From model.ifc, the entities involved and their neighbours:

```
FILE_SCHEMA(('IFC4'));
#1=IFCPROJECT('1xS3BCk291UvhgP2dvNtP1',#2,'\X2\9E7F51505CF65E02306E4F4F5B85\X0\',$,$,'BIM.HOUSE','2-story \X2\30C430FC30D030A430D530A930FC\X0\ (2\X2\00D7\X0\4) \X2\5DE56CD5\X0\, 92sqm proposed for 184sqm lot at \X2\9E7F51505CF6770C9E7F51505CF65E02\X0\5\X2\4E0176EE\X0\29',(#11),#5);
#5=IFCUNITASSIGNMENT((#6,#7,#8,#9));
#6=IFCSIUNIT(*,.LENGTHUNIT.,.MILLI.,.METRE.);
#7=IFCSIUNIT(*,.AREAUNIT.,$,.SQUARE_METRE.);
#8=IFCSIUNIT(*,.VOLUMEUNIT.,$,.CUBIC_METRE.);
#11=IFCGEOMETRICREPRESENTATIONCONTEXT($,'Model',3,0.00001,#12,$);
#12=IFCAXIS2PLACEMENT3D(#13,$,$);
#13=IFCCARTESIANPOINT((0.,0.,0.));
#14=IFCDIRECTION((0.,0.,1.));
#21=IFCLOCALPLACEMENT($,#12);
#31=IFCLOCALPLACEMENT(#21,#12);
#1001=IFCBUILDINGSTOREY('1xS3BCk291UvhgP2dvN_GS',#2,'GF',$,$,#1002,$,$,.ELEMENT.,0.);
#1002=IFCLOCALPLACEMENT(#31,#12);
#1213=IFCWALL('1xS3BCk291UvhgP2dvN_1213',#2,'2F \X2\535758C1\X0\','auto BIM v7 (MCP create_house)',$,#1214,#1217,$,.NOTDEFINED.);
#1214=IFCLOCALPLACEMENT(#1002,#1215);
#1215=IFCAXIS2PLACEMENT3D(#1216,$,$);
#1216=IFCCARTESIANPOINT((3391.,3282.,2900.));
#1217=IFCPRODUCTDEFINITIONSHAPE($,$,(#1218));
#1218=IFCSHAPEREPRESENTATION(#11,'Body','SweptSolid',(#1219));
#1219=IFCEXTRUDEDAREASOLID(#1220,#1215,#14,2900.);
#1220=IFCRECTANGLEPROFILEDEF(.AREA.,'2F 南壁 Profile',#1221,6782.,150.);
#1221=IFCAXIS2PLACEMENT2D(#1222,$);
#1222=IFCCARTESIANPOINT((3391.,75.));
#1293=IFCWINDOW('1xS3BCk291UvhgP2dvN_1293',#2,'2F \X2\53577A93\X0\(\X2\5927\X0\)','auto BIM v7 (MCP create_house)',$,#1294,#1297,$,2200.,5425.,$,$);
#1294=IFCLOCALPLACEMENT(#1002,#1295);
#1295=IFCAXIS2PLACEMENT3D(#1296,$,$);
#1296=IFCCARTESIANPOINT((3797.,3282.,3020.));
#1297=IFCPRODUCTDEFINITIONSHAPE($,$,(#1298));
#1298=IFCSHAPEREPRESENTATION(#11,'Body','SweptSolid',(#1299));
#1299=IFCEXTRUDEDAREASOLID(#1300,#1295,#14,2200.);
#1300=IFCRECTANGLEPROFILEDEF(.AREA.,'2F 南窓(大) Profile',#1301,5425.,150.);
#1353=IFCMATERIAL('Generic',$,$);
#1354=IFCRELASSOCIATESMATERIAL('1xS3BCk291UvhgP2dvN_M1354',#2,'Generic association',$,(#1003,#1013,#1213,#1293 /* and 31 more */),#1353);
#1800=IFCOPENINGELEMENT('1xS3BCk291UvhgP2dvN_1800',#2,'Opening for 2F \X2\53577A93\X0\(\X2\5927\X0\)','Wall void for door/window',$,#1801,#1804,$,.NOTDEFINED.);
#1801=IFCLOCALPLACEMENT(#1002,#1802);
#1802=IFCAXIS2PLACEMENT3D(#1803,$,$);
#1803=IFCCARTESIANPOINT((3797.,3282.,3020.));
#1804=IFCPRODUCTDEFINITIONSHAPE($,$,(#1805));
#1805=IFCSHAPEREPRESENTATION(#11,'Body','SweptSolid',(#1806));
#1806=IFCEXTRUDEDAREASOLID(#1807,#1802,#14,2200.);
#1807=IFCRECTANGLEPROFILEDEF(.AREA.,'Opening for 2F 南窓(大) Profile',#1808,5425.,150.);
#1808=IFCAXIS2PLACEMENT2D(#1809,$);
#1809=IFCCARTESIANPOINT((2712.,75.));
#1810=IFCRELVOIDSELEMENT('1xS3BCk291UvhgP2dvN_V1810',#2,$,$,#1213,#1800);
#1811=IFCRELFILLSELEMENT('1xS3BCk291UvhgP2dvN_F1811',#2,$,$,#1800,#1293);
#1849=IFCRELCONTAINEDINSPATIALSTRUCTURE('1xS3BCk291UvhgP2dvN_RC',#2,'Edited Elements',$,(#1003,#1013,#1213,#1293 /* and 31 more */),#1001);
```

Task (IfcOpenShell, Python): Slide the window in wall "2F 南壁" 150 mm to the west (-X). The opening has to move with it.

```python
import ifcopenshell
import ifcopenshell.api.geometry
import ifcopenshell.util.placement
import ifcopenshell.util.unit

model = ifcopenshell.open("model.ifc")
unit_scale = ifcopenshell.util.unit.calculate_unit_scale(model)

window = model.by_guid("1xS3BCk291UvhgP2dvN_1293")
opening = window.FillsVoids[0].RelatingOpeningElement
wall = opening.VoidsElements[0].RelatingBuildingElement

wall_matrix = ifcopenshell.util.placement.get_local_placement(wall.ObjectPlacement)
shift = wall_matrix[:3, 0] * -0.15 / unit_scale
before = ifcopenshell.util.placement.get_local_placement(window.ObjectPlacement)[:3, 3].copy()

# The window is not placed relative to its opening, so move both.
for product in (opening, window):
    matrix = ifcopenshell.util.placement.get_local_placement(product.ObjectPlacement)
    matrix[:3, 3] += shift
    ifcopenshell.api.geometry.edit_object_placement(model, product=product, matrix=matrix, is_si=False)

after = ifcopenshell.util.placement.get_local_placement(window.ObjectPlacement)[:3, 3]
print("window moved by", (after - before).round(3) + 0.0)

model.write("model_edited.ifc")
```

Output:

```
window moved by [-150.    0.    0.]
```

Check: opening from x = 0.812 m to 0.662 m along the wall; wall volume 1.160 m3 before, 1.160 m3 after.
